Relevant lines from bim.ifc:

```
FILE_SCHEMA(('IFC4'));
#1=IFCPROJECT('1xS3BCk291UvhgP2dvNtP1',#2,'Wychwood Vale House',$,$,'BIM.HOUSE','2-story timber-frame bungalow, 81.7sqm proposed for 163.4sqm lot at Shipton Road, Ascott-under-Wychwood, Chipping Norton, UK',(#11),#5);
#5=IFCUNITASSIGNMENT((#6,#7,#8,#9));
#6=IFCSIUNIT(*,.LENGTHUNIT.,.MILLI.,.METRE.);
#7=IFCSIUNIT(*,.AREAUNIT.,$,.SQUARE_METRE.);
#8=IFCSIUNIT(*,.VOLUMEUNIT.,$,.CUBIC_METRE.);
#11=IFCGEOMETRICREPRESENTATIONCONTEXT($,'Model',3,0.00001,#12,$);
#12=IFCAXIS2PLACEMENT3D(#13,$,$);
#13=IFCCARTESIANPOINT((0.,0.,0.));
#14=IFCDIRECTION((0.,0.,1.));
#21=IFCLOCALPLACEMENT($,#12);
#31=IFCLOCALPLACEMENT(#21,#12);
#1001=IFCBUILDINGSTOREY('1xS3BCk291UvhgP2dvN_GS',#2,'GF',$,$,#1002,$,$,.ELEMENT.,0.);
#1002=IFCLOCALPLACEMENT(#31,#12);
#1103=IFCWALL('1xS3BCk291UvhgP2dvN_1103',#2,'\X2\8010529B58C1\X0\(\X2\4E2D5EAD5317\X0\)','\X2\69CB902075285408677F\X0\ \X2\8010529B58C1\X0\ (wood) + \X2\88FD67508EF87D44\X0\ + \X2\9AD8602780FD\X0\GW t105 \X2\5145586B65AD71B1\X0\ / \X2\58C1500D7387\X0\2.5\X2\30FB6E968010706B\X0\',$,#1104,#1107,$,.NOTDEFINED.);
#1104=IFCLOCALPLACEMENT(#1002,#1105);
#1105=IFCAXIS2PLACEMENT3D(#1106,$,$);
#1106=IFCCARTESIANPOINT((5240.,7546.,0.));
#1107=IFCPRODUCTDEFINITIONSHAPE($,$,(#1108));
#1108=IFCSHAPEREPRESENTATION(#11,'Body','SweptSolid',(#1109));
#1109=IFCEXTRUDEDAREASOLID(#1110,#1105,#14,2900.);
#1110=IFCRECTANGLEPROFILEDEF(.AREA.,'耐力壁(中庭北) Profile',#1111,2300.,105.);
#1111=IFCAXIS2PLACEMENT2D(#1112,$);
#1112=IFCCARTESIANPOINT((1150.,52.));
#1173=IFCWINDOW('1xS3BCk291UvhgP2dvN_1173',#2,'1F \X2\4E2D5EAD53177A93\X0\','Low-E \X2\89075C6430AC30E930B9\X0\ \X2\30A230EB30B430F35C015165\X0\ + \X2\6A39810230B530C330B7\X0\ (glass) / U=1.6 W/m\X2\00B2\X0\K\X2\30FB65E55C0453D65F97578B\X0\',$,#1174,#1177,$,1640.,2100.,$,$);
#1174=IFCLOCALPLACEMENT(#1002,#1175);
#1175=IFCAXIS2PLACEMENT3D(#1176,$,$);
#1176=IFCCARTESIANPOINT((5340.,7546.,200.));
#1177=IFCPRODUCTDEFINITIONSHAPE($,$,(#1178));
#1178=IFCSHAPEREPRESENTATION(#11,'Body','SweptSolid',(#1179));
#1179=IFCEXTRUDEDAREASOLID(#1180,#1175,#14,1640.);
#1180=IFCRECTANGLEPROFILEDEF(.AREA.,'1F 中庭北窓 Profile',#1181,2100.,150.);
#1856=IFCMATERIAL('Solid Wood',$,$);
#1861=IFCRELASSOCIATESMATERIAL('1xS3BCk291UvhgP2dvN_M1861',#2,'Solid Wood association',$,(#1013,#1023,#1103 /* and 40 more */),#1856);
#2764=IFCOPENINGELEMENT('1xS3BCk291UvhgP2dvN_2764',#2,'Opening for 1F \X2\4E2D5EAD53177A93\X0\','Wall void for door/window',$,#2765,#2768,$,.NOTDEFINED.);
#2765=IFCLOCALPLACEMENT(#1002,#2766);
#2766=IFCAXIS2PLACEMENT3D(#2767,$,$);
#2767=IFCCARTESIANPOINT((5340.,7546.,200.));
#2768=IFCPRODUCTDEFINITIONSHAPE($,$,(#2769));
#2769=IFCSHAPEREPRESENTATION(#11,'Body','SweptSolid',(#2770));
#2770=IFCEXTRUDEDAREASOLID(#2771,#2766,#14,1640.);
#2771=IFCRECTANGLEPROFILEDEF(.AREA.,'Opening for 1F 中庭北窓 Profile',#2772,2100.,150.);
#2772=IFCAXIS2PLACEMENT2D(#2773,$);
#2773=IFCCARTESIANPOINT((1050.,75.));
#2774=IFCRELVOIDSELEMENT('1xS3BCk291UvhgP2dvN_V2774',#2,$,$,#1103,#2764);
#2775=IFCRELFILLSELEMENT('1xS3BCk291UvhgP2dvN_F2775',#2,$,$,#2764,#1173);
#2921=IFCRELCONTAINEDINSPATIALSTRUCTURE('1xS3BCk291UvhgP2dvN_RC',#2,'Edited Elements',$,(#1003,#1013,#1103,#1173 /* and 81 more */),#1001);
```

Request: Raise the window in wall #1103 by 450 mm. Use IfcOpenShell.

```python
import numpy as np
import ifcopenshell
import ifcopenshell.api.geometry
import ifcopenshell.util.placement
import ifcopenshell.util.unit

model = ifcopenshell.open("bim.ifc")
unit_scale = ifcopenshell.util.unit.calculate_unit_scale(model)

window = model.by_guid("1xS3BCk291UvhgP2dvN_1173")
opening = window.FillsVoids[0].RelatingOpeningElement
dz = 450.0

shift = np.array([0.0, 0.0, dz])
# The window is not placed relative to its opening, so move both.
for product in (opening, window):
    matrix = ifcopenshell.util.placement.get_local_placement(product.ObjectPlacement)
    matrix[:3, 3] += shift
    ifcopenshell.api.geometry.edit_object_placement(model, product=product, matrix=matrix, is_si=False)

print(f"moved by {dz * unit_scale:+.3f} m")

model.write("bim_edited.ifc")
```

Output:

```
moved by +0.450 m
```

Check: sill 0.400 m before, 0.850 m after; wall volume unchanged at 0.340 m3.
